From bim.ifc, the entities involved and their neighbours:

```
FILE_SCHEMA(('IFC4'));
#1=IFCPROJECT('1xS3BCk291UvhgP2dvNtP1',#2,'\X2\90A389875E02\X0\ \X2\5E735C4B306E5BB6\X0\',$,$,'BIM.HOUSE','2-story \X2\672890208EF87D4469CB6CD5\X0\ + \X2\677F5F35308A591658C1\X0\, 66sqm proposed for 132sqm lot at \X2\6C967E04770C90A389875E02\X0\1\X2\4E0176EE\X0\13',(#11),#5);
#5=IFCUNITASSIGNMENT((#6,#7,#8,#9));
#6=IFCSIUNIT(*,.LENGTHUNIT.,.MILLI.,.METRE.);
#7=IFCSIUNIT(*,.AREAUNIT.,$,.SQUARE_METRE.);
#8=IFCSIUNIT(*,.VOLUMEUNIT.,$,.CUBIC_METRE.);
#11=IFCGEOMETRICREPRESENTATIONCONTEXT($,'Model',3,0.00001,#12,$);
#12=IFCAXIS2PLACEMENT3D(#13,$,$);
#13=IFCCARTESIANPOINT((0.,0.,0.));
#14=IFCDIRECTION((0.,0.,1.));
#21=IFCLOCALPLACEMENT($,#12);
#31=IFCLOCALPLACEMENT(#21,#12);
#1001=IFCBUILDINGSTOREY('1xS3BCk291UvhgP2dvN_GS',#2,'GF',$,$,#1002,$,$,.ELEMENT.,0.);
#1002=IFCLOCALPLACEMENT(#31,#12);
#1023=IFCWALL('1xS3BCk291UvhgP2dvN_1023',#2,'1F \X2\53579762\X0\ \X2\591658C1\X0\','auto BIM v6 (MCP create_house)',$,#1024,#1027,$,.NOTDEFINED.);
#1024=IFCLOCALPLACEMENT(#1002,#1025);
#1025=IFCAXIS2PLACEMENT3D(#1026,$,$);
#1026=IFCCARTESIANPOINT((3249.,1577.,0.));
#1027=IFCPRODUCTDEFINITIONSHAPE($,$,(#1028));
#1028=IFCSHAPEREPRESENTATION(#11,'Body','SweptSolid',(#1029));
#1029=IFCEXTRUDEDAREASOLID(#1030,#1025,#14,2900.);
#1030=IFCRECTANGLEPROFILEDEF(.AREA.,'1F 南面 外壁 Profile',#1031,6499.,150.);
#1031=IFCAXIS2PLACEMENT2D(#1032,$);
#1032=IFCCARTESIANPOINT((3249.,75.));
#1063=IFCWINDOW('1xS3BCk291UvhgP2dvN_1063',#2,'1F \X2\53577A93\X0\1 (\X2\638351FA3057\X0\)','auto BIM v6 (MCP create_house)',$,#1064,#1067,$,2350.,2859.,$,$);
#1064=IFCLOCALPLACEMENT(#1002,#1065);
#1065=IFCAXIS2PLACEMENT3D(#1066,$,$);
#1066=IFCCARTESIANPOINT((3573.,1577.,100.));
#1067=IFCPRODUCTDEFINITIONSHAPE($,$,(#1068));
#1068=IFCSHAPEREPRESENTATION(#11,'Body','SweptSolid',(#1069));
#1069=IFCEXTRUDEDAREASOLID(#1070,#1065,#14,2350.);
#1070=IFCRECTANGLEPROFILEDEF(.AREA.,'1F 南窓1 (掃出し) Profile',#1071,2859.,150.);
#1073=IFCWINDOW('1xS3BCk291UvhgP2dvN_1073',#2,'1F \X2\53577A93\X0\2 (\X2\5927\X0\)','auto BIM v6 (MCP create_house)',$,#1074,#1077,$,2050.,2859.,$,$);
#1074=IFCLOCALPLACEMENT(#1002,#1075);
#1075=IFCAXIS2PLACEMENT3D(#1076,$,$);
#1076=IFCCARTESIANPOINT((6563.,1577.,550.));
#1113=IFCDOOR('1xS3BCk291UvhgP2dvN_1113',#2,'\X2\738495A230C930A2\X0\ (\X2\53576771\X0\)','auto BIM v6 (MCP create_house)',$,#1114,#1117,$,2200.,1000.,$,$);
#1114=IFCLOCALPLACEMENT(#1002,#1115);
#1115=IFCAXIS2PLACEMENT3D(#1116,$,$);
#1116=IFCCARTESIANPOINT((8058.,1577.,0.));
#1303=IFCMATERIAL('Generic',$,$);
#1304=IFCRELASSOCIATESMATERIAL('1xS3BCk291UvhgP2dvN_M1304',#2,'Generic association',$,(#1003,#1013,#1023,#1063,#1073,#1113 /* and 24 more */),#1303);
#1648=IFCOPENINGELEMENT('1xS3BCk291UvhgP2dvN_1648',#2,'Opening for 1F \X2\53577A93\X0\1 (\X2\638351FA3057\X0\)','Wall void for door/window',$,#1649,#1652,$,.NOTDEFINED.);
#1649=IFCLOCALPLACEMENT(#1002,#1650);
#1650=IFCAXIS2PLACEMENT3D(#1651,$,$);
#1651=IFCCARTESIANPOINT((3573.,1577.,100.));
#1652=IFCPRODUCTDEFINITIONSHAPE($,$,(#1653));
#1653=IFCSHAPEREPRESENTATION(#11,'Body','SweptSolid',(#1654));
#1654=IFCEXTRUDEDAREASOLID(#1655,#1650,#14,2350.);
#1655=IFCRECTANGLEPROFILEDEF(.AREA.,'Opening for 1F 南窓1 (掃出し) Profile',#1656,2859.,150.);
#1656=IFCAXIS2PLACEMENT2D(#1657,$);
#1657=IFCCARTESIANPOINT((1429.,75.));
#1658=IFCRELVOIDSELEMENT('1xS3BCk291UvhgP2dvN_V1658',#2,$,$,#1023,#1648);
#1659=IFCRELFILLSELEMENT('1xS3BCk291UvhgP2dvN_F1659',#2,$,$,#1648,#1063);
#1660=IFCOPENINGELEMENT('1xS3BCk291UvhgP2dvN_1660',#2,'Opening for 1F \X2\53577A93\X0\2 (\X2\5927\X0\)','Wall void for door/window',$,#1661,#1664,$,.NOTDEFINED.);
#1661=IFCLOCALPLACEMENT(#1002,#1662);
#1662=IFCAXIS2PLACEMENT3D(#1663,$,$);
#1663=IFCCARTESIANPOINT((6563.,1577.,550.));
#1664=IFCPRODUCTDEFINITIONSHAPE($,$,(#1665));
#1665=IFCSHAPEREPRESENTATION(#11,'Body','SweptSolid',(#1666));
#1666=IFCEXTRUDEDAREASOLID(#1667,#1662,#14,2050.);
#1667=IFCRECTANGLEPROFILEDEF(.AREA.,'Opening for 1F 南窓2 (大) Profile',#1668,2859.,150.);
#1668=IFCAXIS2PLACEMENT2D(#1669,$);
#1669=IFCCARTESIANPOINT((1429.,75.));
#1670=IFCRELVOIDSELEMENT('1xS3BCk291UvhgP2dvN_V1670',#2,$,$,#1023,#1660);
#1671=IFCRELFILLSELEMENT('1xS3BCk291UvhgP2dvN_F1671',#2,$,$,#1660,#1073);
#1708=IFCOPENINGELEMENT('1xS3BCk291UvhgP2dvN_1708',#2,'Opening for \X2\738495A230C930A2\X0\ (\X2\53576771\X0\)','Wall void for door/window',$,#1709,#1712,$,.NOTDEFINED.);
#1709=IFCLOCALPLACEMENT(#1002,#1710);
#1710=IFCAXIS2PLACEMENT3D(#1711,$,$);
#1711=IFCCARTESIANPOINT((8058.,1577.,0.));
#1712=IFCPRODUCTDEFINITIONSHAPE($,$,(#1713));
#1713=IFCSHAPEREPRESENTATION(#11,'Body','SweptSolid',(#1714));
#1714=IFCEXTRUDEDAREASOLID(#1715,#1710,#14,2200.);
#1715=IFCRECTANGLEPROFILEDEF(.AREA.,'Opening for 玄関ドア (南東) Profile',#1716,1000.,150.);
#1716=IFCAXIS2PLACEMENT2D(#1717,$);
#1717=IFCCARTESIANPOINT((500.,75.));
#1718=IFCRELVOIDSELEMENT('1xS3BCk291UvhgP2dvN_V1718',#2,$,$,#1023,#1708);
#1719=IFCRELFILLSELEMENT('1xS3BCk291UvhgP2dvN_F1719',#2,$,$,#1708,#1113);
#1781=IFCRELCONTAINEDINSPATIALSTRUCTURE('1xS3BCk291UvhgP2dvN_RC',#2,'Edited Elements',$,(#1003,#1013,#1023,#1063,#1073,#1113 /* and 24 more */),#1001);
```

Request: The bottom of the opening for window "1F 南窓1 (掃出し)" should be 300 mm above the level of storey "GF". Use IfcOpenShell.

```python
import numpy as np
import ifcopenshell
import ifcopenshell.api.geometry
import ifcopenshell.geom
import ifcopenshell.util.element
import ifcopenshell.util.placement
import ifcopenshell.util.shape
import ifcopenshell.util.unit

model = ifcopenshell.open("bim.ifc")
unit_scale = ifcopenshell.util.unit.calculate_unit_scale(model)

window = model.by_guid("1xS3BCk291UvhgP2dvN_1063")
opening = window.FillsVoids[0].RelatingOpeningElement
storey = ifcopenshell.util.element.get_container(window, ifc_class="IfcBuildingStorey")
level = ifcopenshell.util.placement.get_local_placement(storey.ObjectPlacement)[2, 3]

# The opening's origin need not be at the sill, so measure its lowest point.
shape = ifcopenshell.geom.create_shape(ifcopenshell.geom.settings(), opening)
bottom = ifcopenshell.util.shape.get_shape_bottom_elevation(shape, shape.geometry) / unit_scale
dz = level + 300.0 - bottom

shift = np.array([0.0, 0.0, dz])
# The window is not placed relative to its opening, so move both.
for product in (opening, window):
    matrix = ifcopenshell.util.placement.get_local_placement(product.ObjectPlacement)
    matrix[:3, 3] += shift
    ifcopenshell.api.geometry.edit_object_placement(model, product=product, matrix=matrix, is_si=False)

print(f"moved by {dz * unit_scale:+.3f} m")

model.write("bim_rev.ifc")
```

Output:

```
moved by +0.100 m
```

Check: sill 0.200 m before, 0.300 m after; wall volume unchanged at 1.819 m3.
